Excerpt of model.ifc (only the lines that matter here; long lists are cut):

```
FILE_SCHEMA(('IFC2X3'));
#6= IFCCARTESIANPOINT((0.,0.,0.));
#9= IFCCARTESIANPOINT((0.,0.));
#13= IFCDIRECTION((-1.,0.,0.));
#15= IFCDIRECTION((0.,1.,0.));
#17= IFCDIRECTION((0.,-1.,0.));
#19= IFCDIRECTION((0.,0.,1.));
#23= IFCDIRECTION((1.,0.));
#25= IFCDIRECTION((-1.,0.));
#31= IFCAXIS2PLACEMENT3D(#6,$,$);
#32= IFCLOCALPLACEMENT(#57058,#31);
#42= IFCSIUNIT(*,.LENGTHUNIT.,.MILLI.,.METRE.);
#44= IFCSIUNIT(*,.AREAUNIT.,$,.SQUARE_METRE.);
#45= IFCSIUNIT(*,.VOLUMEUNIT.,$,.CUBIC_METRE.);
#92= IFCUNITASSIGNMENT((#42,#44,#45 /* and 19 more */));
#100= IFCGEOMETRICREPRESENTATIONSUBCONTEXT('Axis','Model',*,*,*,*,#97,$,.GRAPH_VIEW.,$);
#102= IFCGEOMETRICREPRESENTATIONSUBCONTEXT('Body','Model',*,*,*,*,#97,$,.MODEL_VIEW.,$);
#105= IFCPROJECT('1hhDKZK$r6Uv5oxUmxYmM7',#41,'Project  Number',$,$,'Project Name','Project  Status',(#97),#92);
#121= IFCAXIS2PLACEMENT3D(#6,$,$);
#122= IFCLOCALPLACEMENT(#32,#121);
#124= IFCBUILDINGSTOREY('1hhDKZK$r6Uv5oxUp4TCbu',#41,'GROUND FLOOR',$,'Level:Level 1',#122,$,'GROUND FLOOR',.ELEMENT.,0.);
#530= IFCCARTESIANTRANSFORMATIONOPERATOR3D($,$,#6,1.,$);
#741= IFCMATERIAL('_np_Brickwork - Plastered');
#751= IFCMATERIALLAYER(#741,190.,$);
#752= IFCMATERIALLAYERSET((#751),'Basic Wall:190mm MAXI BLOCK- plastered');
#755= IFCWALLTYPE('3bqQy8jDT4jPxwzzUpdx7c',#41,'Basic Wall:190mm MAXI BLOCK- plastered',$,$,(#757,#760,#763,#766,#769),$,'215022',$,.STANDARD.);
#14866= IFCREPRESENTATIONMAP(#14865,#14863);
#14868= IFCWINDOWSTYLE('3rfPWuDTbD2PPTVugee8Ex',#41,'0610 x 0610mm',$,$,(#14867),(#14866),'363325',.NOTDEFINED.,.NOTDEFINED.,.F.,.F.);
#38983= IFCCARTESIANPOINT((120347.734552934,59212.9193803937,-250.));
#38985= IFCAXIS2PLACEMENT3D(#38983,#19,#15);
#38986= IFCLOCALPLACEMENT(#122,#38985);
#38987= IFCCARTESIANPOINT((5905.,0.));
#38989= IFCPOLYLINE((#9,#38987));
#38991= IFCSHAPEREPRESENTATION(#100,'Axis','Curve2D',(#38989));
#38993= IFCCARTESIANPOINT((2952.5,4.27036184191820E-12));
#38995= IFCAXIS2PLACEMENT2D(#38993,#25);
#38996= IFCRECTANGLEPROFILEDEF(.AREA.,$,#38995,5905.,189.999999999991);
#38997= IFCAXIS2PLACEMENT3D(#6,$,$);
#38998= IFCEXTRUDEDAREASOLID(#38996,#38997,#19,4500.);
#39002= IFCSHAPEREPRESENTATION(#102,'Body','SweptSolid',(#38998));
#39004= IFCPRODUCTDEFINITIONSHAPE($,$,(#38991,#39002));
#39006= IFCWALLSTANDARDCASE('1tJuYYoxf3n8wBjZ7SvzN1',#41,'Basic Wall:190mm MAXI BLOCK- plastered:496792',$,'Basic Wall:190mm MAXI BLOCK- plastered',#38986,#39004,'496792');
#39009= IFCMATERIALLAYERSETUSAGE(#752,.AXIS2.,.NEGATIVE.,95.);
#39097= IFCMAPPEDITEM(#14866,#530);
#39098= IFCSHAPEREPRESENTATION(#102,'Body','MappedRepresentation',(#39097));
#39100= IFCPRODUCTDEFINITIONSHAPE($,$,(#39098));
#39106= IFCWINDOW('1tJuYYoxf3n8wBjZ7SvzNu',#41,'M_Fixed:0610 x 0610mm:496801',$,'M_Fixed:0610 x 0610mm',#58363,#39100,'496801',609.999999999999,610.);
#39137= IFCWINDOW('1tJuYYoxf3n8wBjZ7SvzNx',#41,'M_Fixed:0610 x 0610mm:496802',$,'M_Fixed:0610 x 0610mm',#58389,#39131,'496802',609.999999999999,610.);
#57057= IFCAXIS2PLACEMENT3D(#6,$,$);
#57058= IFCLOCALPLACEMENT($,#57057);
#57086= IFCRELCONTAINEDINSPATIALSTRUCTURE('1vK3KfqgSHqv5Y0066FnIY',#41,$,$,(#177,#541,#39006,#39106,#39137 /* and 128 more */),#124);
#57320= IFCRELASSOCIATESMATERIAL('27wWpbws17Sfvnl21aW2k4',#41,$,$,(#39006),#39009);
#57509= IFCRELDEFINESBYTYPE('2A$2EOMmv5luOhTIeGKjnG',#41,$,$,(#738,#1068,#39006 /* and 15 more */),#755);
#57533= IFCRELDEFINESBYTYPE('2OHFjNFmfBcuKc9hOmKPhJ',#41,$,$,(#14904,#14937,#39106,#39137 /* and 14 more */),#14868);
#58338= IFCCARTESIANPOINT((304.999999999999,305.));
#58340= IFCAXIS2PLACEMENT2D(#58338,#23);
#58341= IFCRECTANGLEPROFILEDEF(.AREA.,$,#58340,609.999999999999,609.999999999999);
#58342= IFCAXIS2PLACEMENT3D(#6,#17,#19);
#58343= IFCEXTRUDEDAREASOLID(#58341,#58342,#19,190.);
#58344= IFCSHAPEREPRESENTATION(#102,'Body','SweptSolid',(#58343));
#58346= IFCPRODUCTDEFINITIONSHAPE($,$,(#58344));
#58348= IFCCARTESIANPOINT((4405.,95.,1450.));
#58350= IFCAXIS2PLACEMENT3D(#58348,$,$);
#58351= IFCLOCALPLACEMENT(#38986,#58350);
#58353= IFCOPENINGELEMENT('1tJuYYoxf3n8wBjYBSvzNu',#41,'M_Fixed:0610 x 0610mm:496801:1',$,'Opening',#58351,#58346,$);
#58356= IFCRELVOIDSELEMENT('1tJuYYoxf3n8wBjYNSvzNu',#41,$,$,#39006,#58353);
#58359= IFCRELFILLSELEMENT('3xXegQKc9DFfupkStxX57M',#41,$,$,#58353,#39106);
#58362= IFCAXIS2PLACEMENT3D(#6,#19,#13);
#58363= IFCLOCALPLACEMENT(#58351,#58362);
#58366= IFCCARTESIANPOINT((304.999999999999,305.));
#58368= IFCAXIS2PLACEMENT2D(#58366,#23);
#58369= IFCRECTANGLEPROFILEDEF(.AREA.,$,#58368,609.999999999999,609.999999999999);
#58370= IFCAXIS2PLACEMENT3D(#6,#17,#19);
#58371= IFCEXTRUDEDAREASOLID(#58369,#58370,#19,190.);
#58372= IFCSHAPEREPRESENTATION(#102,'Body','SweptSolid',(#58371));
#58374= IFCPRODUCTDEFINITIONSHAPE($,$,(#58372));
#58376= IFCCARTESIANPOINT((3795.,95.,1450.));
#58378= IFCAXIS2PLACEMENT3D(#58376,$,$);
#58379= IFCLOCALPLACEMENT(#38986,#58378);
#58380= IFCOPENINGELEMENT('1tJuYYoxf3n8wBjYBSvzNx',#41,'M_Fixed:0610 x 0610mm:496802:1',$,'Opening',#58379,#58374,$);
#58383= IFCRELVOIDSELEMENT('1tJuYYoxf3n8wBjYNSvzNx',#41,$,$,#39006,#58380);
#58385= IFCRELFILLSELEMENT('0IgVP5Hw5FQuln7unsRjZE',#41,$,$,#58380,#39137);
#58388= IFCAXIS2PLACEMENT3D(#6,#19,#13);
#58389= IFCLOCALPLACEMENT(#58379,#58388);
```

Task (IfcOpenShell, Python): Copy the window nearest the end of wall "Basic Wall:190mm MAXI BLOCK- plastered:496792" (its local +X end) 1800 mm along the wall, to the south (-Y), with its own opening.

```python
import ifcopenshell
import ifcopenshell.api.feature
import ifcopenshell.api.geometry
import ifcopenshell.api.root
import ifcopenshell.geom
import ifcopenshell.util.element
import ifcopenshell.util.placement
import ifcopenshell.util.shape

model = ifcopenshell.open("model.ifc")
settings = ifcopenshell.geom.settings()


def volume(element):
    """Net volume in cubic metres, openings subtracted."""
    shape = ifcopenshell.geom.create_shape(settings, element)
    return ifcopenshell.util.shape.get_volume(shape.geometry)


def reuse_history(source, copy):
    """copy_class also copies each property set's owner history, people and application; keep the originals."""
    for rel in copy.IsDefinedBy:
        if rel.is_a("IfcRelDefinesByProperties") and (history := rel.RelatingPropertyDefinition.OwnerHistory):
            rel.RelatingPropertyDefinition.OwnerHistory = source.OwnerHistory
            ifcopenshell.util.element.remove_deep2(model, history)


window = model.by_id(39106)
opening = window.FillsVoids[0].RelatingOpeningElement
wall = opening.VoidsElements[0].RelatingBuildingElement
before = volume(wall)
shift = ifcopenshell.util.placement.get_local_placement(wall.ObjectPlacement)[:3, 0] * -1800.0

# copy_class copies the void relationship, type, container and properties, but no geometry.
new_opening = ifcopenshell.api.root.copy_class(model, product=opening)
new_opening.Representation = ifcopenshell.util.element.copy_deep(
    model, opening.Representation, exclude=["IfcGeometricRepresentationContext", "IfcRepresentationMap"]
)
new_opening.Name = "M_Fixed:0610 x 0610mm"
new_window = ifcopenshell.api.root.copy_class(model, product=window)
new_window.Representation = ifcopenshell.util.element.copy_deep(
    model, window.Representation, exclude=["IfcGeometricRepresentationContext", "IfcRepresentationMap"]
)
new_window.Name = "M_Fixed:0610 x 0610mm"
new_window.Tag = None
reuse_history(window, new_window)
fills = ifcopenshell.api.feature.add_filling(model, opening=new_opening, element=new_window)
fills.OwnerHistory = new_window.OwnerHistory  # required in IFC2X3

for old, new in ((opening, new_opening), (window, new_window)):
    matrix = ifcopenshell.util.placement.get_local_placement(old.ObjectPlacement)
    matrix[:3, 3] += shift
    ifcopenshell.api.geometry.edit_object_placement(model, product=new, matrix=matrix, is_si=False)

after = volume(wall)

print(f"wall volume {before:.3f} -> {after:.3f} m3")

model.write("model_edited.ifc")
```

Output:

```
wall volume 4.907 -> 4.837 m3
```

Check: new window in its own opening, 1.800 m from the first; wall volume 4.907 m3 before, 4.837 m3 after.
